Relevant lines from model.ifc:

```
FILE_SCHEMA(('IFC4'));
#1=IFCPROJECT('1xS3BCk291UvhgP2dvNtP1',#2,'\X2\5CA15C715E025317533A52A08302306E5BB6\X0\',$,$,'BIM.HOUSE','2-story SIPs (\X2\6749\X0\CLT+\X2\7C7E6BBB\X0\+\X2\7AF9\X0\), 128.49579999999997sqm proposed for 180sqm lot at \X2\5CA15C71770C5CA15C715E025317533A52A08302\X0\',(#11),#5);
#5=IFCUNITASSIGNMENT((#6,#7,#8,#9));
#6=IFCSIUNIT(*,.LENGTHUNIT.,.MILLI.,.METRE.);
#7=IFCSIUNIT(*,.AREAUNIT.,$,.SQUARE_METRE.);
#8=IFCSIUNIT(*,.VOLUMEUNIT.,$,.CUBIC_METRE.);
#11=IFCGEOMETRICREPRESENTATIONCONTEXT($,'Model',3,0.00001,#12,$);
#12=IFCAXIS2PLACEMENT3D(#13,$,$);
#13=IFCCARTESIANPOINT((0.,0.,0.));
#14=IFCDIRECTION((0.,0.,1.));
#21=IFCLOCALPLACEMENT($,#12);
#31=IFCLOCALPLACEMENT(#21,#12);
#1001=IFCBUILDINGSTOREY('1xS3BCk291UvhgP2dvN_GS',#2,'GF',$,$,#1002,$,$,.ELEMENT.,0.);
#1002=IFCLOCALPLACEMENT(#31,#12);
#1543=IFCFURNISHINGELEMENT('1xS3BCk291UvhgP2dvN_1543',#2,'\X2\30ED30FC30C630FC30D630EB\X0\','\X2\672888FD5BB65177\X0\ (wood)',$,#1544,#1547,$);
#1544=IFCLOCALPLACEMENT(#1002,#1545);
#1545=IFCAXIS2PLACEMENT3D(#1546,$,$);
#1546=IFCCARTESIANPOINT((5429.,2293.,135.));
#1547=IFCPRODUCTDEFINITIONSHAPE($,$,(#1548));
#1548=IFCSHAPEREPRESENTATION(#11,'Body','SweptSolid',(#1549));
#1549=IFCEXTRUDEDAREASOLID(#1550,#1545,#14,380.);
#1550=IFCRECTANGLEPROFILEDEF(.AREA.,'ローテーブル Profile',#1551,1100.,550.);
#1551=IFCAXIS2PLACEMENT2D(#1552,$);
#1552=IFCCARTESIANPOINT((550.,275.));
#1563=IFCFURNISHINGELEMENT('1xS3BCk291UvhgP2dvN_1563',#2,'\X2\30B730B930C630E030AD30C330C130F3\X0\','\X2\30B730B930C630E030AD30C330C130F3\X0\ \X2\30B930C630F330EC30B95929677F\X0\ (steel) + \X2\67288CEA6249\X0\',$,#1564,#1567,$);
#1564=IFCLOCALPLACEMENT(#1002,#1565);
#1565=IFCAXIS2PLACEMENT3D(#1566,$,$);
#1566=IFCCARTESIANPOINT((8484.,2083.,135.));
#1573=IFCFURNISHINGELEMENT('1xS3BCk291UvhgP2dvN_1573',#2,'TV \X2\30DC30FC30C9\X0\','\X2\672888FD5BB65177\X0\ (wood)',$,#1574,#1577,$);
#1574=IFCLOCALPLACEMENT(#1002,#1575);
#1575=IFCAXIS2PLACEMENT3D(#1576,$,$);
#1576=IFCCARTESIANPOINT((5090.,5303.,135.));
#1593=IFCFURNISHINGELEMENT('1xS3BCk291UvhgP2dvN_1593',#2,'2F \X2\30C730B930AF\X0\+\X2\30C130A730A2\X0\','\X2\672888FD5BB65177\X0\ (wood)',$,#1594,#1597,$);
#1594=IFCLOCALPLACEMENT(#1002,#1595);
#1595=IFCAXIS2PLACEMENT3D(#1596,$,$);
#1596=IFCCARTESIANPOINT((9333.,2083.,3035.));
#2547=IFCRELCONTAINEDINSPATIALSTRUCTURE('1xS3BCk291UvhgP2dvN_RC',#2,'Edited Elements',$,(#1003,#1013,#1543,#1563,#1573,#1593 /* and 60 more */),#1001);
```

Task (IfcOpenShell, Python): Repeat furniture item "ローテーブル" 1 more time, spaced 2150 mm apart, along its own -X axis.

```python
import ifcopenshell
import ifcopenshell.api.geometry
import ifcopenshell.api.root
import ifcopenshell.util.element
import ifcopenshell.util.placement
import ifcopenshell.util.unit

model = ifcopenshell.open("model.ifc")
unit_scale = ifcopenshell.util.unit.calculate_unit_scale(model)


def reuse_history(source, copy):
    """copy_class also copies each property set's owner history, people and application; keep the originals."""
    for rel in copy.IsDefinedBy:
        if rel.is_a("IfcRelDefinesByProperties") and (history := rel.RelatingPropertyDefinition.OwnerHistory):
            rel.RelatingPropertyDefinition.OwnerHistory = source.OwnerHistory
            ifcopenshell.util.element.remove_deep2(model, history)


source = model.by_guid("1xS3BCk291UvhgP2dvN_1543")
base = ifcopenshell.util.placement.get_local_placement(source.ObjectPlacement)
step = -base[:3, 0] * 2.15 / unit_scale

for i in range(1, 2):
    copy = ifcopenshell.api.root.copy_class(model, product=source)
    copy.Representation = ifcopenshell.util.element.copy_deep(
        model, source.Representation, exclude=["IfcGeometricRepresentationContext", "IfcRepresentationMap"]
    )
    reuse_history(source, copy)
    matrix = base.copy()
    matrix[:3, 3] += i * step
    print("added at", matrix[:3, 3].round(3) + 0.0)
    ifcopenshell.api.geometry.edit_object_placement(model, product=copy, matrix=matrix, is_si=False)

model.write("model_rev.ifc")
```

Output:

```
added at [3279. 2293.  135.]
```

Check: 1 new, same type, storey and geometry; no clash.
